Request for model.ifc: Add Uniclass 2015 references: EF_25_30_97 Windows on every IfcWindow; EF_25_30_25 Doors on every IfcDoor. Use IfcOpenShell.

First a look at what the model holds.

```python
import ifcopenshell

model = ifcopenshell.open("model.ifc")
print(model.schema)
print("classifications:", [c.Name for c in model.by_type("IfcClassification")])
for ifc_class in ("IfcDoor", "IfcRoof", "IfcStair", "IfcWall", "IfcWindow"):
    print(ifc_class, len(model.by_type(ifc_class)))
```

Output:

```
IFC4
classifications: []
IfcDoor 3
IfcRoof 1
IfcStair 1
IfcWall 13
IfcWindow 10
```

```python
import ifcopenshell
import ifcopenshell.api.classification

model = ifcopenshell.open("model.ifc")

system = ifcopenshell.api.classification.add_classification(model, classification="Uniclass 2015")

codes = {
    "IfcWindow": ("EF_25_30_97", "Windows"),
    "IfcDoor": ("EF_25_30_25", "Doors"),
}
for ifc_class, (code, name) in codes.items():
    products = model.by_type(ifc_class)
    ifcopenshell.api.classification.add_reference(
        model, products=products, classification=system, identification=code, name=name
    )
    print(code, len(products))

model.write("model_v2.ifc")
```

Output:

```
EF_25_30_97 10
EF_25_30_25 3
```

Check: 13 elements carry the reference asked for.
